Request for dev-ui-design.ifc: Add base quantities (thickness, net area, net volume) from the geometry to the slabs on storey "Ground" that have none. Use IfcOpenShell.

First a look at what the model holds.

```python
import ifcopenshell
import ifcopenshell.util.element
import ifcopenshell.util.unit

model = ifcopenshell.open("dev-ui-design.ifc")
print(model.schema)
for unit_type in ("LENGTHUNIT", "AREAUNIT", "VOLUMEUNIT"):
    print(unit_type, ifcopenshell.util.unit.calculate_unit_scale(model, unit_type))
storey = next(s for s in model.by_type("IfcBuildingStorey") if s.Name == "Ground")
slabs = [e for e in ifcopenshell.util.element.get_decomposition(storey) if e.is_a("IfcSlab")]
for e in sorted(slabs, key=lambda e: e.id()):
    print(e.id(), e.is_a(), e.Name, list(ifcopenshell.util.element.get_psets(e, qtos_only=True)), sep=" | ")
```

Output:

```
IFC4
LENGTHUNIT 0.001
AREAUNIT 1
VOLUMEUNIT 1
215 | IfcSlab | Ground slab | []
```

```python
import ifcopenshell
import ifcopenshell.api.pset
import ifcopenshell.geom
import ifcopenshell.util.element
import ifcopenshell.util.shape
import ifcopenshell.util.unit

model = ifcopenshell.open("dev-ui-design.ifc")
unit_scale = ifcopenshell.util.unit.calculate_unit_scale(model)
area_scale = ifcopenshell.util.unit.calculate_unit_scale(model, "AREAUNIT")
volume_scale = ifcopenshell.util.unit.calculate_unit_scale(model, "VOLUMEUNIT")
settings = ifcopenshell.geom.settings()

storey = next(s for s in model.by_type("IfcBuildingStorey") if s.Name == "Ground")
slabs = [e for e in ifcopenshell.util.element.get_decomposition(storey) if e.is_a("IfcSlab")]

for e in sorted(slabs, key=lambda e: e.id()):
    if ifcopenshell.util.element.get_psets(e, qtos_only=True, should_inherit=False):
        continue
    # Geometry comes back in metres, in the element's own axes.
    shape = ifcopenshell.geom.create_shape(settings, e)
    values = {
        "Width": ifcopenshell.util.shape.get_z(shape.geometry) / unit_scale,
        "NetArea": ifcopenshell.util.shape.get_footprint_area(shape.geometry) / area_scale,
        "NetVolume": ifcopenshell.util.shape.get_volume(shape.geometry) / volume_scale,
    }
    qto = ifcopenshell.api.pset.add_qto(model, product=e, name="Qto_SlabBaseQuantities")
    ifcopenshell.api.pset.edit_qto(model, qto=qto, properties=values)
    print(e.id(), {k: round(v, 3) for k, v in values.items()})

model.write("dev-ui-design-out.ifc")
```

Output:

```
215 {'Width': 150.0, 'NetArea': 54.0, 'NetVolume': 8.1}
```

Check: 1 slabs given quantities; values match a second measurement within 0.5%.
